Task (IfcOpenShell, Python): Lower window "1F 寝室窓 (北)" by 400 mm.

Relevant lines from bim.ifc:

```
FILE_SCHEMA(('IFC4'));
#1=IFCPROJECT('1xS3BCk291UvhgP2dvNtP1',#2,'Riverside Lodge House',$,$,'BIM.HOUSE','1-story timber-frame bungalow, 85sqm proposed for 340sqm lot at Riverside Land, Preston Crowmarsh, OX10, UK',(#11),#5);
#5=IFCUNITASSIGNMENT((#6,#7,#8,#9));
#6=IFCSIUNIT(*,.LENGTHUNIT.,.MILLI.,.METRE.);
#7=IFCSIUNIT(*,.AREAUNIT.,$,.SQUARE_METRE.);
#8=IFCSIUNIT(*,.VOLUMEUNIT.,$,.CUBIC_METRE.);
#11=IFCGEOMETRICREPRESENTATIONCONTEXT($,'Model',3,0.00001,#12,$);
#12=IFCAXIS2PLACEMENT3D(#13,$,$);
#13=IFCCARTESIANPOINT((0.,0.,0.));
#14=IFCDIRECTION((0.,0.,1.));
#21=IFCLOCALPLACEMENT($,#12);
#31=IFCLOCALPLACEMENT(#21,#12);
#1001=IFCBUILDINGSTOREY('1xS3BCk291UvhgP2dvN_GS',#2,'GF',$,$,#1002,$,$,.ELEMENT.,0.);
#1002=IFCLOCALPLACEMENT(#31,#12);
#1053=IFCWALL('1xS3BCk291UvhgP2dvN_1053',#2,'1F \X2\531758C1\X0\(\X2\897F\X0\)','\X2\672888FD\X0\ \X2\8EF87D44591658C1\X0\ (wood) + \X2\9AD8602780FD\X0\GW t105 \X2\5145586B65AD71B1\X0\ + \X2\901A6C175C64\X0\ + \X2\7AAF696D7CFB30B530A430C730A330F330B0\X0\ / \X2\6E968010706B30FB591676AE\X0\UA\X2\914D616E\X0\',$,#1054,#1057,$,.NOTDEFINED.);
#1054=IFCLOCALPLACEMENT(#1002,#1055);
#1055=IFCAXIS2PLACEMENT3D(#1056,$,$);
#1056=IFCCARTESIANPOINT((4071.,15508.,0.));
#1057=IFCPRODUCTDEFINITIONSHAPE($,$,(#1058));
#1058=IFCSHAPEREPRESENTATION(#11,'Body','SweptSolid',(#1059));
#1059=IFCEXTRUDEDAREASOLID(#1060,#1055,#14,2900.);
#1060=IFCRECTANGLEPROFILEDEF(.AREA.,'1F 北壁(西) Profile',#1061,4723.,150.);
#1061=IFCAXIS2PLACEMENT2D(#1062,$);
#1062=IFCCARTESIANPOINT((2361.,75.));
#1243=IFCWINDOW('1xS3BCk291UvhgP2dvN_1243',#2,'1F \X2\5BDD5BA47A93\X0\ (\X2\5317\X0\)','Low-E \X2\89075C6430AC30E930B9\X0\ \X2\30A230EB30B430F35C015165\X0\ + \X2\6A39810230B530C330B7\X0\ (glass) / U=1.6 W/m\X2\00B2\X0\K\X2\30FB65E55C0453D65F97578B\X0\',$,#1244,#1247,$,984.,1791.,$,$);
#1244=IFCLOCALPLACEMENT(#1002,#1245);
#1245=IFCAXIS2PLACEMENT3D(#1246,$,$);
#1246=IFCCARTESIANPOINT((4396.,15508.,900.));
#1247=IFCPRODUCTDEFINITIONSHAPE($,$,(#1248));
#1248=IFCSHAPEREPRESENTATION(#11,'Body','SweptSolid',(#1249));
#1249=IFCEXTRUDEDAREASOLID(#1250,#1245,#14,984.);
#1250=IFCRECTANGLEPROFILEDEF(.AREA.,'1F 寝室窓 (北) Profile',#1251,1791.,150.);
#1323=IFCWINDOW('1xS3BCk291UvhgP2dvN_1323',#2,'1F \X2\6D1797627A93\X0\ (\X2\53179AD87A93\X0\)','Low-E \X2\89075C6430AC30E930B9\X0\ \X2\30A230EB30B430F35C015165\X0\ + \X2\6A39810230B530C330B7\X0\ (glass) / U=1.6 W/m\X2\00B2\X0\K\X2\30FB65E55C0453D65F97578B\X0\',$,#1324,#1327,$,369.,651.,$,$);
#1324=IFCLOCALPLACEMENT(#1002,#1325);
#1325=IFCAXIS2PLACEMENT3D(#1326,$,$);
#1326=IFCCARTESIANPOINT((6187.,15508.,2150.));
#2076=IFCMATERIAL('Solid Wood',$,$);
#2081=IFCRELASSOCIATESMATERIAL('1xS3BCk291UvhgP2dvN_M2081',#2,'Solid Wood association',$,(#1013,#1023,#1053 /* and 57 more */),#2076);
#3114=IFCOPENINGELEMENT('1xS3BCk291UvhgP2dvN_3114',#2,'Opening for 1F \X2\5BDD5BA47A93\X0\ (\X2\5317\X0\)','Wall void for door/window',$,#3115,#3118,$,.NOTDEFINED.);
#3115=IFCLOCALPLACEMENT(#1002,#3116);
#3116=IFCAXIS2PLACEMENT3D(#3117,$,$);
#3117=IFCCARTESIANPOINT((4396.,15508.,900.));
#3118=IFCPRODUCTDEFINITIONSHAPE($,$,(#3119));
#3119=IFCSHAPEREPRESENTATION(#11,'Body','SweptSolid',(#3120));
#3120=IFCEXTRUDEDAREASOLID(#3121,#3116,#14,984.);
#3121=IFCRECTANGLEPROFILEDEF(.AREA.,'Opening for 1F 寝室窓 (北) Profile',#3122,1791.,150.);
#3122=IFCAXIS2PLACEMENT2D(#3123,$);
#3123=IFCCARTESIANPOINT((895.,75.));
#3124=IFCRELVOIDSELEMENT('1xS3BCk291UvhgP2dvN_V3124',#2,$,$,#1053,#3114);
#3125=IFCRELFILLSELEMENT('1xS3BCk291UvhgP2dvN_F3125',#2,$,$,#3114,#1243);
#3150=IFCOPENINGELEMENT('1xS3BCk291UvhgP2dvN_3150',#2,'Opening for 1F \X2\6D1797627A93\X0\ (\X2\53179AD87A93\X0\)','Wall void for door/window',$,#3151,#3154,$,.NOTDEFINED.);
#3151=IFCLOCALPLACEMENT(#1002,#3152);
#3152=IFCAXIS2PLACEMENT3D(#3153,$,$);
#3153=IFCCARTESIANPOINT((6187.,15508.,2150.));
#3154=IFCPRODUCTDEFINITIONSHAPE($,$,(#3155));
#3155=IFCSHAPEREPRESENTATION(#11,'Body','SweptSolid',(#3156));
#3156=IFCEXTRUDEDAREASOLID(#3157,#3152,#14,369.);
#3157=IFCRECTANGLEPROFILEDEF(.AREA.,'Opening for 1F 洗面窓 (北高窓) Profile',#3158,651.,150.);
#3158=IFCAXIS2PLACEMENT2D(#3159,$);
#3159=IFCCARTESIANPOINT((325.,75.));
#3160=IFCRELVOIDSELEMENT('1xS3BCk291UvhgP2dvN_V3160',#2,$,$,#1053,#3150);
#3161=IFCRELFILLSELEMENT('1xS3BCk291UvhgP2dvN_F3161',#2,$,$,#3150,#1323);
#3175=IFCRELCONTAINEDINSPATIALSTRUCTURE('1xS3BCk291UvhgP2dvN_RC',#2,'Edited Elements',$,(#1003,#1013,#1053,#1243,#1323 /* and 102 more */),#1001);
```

```python
import numpy as np
import ifcopenshell
import ifcopenshell.api.geometry
import ifcopenshell.util.placement
import ifcopenshell.util.unit

model = ifcopenshell.open("bim.ifc")
unit_scale = ifcopenshell.util.unit.calculate_unit_scale(model)

window = model.by_guid("1xS3BCk291UvhgP2dvN_1243")
opening = window.FillsVoids[0].RelatingOpeningElement
dz = -0.4 / unit_scale

shift = np.array([0.0, 0.0, dz])
# The window is not placed relative to its opening, so move both.
for product in (opening, window):
    matrix = ifcopenshell.util.placement.get_local_placement(product.ObjectPlacement)
    matrix[:3, 3] += shift
    ifcopenshell.api.geometry.edit_object_placement(model, product=product, matrix=matrix, is_si=False)

print(f"moved by {dz * unit_scale:+.3f} m")

model.write("bim_rev.ifc")
```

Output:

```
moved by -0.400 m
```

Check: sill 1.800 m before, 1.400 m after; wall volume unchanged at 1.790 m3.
